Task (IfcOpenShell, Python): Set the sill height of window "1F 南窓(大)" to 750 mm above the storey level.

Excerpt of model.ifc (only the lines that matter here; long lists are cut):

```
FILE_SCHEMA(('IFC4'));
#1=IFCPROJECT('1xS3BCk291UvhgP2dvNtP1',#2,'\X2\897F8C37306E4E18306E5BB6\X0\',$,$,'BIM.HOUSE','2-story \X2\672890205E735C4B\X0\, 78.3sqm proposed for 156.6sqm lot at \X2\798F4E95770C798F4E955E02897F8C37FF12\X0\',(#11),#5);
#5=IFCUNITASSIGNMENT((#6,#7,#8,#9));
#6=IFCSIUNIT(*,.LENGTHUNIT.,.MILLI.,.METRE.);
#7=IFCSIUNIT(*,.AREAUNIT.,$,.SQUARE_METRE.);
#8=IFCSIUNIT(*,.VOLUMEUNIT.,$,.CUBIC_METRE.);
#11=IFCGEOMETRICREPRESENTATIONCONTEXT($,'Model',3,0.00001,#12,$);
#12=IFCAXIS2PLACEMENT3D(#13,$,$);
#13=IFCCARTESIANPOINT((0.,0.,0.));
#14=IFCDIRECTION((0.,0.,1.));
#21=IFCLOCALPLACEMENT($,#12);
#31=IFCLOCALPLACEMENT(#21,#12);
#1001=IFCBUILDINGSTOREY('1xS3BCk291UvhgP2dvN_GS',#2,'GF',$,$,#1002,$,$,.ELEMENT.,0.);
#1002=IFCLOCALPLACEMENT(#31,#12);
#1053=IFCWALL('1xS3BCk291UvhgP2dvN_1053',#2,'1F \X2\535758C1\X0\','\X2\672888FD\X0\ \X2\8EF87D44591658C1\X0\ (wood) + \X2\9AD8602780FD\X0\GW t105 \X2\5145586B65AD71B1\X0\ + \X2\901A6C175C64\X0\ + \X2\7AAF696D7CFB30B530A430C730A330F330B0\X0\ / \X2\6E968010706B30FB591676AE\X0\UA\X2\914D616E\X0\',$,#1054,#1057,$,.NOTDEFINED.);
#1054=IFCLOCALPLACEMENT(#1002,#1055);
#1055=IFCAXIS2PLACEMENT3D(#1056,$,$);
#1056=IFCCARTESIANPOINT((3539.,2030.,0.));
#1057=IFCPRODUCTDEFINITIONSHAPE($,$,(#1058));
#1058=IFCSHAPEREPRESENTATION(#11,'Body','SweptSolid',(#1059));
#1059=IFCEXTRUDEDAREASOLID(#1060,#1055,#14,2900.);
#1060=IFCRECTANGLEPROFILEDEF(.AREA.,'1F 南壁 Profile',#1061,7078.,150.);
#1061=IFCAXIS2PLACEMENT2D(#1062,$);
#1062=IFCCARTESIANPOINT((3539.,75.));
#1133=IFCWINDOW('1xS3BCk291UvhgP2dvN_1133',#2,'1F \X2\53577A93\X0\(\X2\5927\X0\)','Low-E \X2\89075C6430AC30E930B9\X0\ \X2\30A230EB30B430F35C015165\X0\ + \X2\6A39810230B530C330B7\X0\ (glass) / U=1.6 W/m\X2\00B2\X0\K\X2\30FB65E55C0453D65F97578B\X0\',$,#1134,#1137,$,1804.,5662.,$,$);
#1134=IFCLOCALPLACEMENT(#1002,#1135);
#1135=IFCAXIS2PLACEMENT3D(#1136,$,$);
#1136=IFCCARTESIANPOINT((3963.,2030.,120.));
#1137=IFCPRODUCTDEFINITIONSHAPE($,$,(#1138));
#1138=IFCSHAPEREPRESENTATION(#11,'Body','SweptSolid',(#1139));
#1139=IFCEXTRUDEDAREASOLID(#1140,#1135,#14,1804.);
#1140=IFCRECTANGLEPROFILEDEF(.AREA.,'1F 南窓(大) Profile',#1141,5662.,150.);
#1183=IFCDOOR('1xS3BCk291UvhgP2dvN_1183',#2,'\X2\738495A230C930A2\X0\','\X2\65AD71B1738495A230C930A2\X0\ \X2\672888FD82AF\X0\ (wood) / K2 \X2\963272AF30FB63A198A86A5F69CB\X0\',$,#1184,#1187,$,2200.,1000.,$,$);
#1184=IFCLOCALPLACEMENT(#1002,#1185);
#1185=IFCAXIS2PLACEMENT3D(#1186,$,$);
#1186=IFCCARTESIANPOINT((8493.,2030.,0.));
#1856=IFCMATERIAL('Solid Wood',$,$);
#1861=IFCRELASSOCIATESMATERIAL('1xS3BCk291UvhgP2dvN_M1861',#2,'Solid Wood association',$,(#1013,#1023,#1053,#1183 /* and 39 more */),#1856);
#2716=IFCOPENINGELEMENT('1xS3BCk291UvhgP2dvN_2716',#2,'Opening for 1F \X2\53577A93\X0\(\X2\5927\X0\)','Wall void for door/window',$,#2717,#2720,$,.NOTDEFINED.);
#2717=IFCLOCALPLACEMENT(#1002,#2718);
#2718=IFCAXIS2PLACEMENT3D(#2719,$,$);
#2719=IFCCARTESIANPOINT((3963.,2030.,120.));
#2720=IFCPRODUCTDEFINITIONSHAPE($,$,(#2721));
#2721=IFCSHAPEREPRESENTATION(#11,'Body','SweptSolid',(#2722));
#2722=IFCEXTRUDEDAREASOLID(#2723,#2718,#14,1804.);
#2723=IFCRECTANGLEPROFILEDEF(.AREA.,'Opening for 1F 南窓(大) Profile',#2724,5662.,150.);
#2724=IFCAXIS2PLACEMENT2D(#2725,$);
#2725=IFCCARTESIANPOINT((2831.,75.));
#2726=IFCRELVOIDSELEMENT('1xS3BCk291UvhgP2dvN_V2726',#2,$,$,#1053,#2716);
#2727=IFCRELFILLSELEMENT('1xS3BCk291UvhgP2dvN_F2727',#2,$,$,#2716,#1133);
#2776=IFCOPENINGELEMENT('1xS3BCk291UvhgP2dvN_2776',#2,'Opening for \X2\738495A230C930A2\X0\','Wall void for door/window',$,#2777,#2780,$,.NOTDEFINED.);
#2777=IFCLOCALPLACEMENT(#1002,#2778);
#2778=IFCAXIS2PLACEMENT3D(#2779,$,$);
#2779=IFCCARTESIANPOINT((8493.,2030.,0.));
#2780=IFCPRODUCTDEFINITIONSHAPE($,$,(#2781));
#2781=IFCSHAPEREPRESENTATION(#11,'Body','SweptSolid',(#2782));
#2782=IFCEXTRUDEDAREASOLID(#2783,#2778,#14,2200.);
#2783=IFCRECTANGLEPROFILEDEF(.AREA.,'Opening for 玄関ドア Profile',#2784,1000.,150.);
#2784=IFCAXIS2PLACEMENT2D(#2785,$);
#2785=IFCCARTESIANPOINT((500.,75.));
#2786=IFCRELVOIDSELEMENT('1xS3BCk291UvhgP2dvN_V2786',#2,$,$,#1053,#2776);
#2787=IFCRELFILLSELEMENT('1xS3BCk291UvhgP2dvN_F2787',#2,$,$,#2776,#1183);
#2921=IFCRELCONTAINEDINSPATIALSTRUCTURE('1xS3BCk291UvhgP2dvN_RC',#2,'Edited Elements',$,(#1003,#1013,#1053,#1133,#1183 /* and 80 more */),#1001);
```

```python
import numpy as np
import ifcopenshell
import ifcopenshell.api.geometry
import ifcopenshell.geom
import ifcopenshell.util.element
import ifcopenshell.util.placement
import ifcopenshell.util.shape
import ifcopenshell.util.unit

model = ifcopenshell.open("model.ifc")
unit_scale = ifcopenshell.util.unit.calculate_unit_scale(model)

window = model.by_guid("1xS3BCk291UvhgP2dvN_1133")
opening = window.FillsVoids[0].RelatingOpeningElement
storey = ifcopenshell.util.element.get_container(window, ifc_class="IfcBuildingStorey")
level = ifcopenshell.util.placement.get_local_placement(storey.ObjectPlacement)[2, 3]

# The opening's origin need not be at the sill, so measure its lowest point.
shape = ifcopenshell.geom.create_shape(ifcopenshell.geom.settings(), opening)
bottom = ifcopenshell.util.shape.get_shape_bottom_elevation(shape, shape.geometry) / unit_scale
dz = level + 0.75 / unit_scale - bottom

shift = np.array([0.0, 0.0, dz])
# The window is not placed relative to its opening, so move both.
for product in (opening, window):
    matrix = ifcopenshell.util.placement.get_local_placement(product.ObjectPlacement)
    matrix[:3, 3] += shift
    ifcopenshell.api.geometry.edit_object_placement(model, product=product, matrix=matrix, is_si=False)

print(f"moved by {dz * unit_scale:+.3f} m")

model.write("model_edited.ifc")
```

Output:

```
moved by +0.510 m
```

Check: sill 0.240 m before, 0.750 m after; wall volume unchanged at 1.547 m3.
